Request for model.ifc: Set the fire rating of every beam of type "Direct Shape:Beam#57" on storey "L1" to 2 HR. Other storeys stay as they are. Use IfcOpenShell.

First a look at what the model holds.

```python
import ifcopenshell
import ifcopenshell.util.element

model = ifcopenshell.open("model.ifc")
print(model.schema)
storey = next(s for s in model.by_type("IfcBuildingStorey") if s.Name == "L1")
beams = [e for e in ifcopenshell.util.element.get_decomposition(storey) if e.is_a("IfcBeam")]
seen = {}
for e in beams:
    element_type = ifcopenshell.util.element.get_type(e)
    key = (element_type.Name if element_type != e and element_type else None, ifcopenshell.util.element.get_pset(e, "Pset_BeamCommon", "FireRating"))
    seen[key] = seen.get(key, 0) + 1
for (name, value), count in sorted(seen.items(), key=str):
    print(count, "x", name, "|", value)
```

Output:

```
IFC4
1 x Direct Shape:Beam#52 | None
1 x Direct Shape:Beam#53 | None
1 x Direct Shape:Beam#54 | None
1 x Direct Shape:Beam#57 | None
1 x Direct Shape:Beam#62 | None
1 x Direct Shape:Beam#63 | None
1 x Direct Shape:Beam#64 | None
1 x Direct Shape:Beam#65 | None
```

```python
import ifcopenshell
import ifcopenshell.api.pset
import ifcopenshell.util.element

model = ifcopenshell.open("model.ifc")

storey = next(s for s in model.by_type("IfcBuildingStorey") if s.Name == "L1")
beams = [e for e in ifcopenshell.util.element.get_decomposition(storey) if e.is_a("IfcBeam")]

count = 0
for e in beams:
    element_type = ifcopenshell.util.element.get_type(e)
    if element_type in (None, e) or element_type.Name != "Direct Shape:Beam#57":
        continue
    # add_pset returns the element's existing set when there is one.
    pset = ifcopenshell.api.pset.add_pset(model, product=e, name="Pset_BeamCommon")
    ifcopenshell.api.pset.edit_pset(model, pset=pset, properties={"FireRating": "2 HR"})
    count += 1

print(count, "beams updated")

model.write("model-out.ifc")
```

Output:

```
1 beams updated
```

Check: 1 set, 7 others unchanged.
